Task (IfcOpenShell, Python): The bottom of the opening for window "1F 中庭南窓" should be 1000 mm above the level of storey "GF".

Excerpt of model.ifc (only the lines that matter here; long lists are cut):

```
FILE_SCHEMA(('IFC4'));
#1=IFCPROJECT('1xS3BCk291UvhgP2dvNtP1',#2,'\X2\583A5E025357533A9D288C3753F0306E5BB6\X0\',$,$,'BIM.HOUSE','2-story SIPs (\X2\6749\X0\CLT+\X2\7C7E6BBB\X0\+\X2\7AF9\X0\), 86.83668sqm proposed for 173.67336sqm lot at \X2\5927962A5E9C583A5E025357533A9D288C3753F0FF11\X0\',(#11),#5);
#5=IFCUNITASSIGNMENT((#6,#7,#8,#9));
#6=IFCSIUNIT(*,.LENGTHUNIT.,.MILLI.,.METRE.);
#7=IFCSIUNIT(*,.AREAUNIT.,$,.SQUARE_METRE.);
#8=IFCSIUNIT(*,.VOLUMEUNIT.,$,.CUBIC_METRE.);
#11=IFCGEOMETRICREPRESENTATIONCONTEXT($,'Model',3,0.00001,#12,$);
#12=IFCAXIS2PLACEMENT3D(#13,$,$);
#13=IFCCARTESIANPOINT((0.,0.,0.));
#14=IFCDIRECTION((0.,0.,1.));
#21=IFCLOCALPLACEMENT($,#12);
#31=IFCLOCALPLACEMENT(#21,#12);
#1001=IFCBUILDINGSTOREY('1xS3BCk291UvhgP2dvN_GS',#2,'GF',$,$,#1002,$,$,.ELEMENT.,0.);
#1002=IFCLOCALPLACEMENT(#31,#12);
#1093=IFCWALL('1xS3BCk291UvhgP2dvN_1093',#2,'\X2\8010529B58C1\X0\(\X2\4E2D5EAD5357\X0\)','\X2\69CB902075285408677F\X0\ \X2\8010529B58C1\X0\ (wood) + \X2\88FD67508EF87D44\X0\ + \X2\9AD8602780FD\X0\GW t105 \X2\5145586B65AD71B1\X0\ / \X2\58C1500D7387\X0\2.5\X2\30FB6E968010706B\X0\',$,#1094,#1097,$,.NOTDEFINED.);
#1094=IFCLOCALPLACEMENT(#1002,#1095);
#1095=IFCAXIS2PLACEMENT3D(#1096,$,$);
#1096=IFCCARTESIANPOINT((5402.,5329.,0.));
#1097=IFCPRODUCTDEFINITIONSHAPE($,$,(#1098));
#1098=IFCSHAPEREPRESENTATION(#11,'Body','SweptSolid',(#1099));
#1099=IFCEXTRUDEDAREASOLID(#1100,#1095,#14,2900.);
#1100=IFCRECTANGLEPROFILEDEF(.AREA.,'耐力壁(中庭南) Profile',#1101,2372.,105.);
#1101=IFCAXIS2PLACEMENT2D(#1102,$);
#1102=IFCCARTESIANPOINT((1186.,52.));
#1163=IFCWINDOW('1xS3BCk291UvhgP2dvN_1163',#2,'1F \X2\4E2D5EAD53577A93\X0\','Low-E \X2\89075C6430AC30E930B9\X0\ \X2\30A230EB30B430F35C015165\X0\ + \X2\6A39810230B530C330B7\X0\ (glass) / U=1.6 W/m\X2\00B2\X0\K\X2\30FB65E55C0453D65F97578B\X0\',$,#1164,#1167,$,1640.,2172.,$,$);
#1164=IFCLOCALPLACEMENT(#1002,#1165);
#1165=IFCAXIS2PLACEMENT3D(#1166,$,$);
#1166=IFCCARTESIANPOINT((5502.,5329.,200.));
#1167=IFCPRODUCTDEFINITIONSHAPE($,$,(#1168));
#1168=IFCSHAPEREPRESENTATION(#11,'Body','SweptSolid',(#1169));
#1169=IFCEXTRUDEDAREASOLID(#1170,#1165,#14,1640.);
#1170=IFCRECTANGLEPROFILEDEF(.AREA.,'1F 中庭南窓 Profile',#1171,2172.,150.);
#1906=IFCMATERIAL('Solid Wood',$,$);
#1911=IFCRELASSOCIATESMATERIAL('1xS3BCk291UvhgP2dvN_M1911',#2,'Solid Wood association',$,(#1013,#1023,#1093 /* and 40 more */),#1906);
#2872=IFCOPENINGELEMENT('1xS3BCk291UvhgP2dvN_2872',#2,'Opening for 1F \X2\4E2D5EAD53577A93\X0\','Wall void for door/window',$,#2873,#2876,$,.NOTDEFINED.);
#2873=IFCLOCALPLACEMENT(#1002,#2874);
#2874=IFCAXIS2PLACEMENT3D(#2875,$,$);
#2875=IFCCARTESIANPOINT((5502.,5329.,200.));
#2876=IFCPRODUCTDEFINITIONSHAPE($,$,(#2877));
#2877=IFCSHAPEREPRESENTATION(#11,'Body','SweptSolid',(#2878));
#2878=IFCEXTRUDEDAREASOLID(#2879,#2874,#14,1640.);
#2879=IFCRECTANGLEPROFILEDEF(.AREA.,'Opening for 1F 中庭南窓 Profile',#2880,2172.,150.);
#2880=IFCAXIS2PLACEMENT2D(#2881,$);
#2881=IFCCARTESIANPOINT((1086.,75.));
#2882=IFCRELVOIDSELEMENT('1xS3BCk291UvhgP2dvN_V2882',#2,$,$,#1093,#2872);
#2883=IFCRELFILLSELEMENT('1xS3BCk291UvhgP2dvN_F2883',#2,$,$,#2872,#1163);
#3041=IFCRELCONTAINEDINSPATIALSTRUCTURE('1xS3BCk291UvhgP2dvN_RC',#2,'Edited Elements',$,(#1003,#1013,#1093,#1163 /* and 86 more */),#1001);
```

```python
import numpy as np
import ifcopenshell
import ifcopenshell.api.geometry
import ifcopenshell.geom
import ifcopenshell.util.element
import ifcopenshell.util.placement
import ifcopenshell.util.shape
import ifcopenshell.util.unit

model = ifcopenshell.open("model.ifc")
unit_scale = ifcopenshell.util.unit.calculate_unit_scale(model)

window = model.by_guid("1xS3BCk291UvhgP2dvN_1163")
opening = window.FillsVoids[0].RelatingOpeningElement
storey = ifcopenshell.util.element.get_container(window, ifc_class="IfcBuildingStorey")
level = ifcopenshell.util.placement.get_local_placement(storey.ObjectPlacement)[2, 3]

# The opening's origin need not be at the sill, so measure its lowest point.
shape = ifcopenshell.geom.create_shape(ifcopenshell.geom.settings(), opening)
bottom = ifcopenshell.util.shape.get_shape_bottom_elevation(shape, shape.geometry) / unit_scale
dz = level + 1000.0 - bottom

shift = np.array([0.0, 0.0, dz])
# The window is not placed relative to its opening, so move both.
for product in (opening, window):
    matrix = ifcopenshell.util.placement.get_local_placement(product.ObjectPlacement)
    matrix[:3, 3] += shift
    ifcopenshell.api.geometry.edit_object_placement(model, product=product, matrix=matrix, is_si=False)

print(f"moved by {dz * unit_scale:+.3f} m")

model.write("model_updated.ifc")
```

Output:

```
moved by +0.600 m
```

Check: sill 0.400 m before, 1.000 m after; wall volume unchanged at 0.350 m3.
